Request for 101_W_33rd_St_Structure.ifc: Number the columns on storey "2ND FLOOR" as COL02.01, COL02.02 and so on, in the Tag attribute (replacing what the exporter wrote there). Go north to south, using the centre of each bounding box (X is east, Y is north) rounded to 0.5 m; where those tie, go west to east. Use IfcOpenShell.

First a look at what the model holds.

```python
import ifcopenshell
import ifcopenshell.util.element
import ifcopenshell.util.placement

model = ifcopenshell.open("101_W_33rd_St_Structure.ifc")
print(model.schema)
storey = next(s for s in model.by_type("IfcBuildingStorey") if s.Name == "2ND FLOOR")
columns = [e for e in ifcopenshell.util.element.get_decomposition(storey) if e.is_a("IfcColumn")]
for e in sorted(columns, key=lambda e: e.id()):
    origin = ifcopenshell.util.placement.get_local_placement(e.ObjectPlacement)[:3, 3]
    print(e.id(), e.Tag, e.Name, origin.round(2) + 0.0, sep=" | ")
```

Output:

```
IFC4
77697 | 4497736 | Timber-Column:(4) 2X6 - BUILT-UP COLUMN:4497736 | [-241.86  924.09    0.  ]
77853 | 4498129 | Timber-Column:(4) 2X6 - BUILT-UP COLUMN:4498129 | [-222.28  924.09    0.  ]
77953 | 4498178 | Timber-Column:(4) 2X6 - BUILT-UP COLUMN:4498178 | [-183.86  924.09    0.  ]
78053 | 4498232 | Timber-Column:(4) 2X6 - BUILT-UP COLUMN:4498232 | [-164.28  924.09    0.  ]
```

```python
import ifcopenshell
import ifcopenshell.geom
import ifcopenshell.util.element
import ifcopenshell.util.shape

model = ifcopenshell.open("101_W_33rd_St_Structure.ifc")
settings = ifcopenshell.geom.settings()
settings.set("use-world-coords", True)


def centre(element):
    shape = ifcopenshell.geom.create_shape(settings, element)
    return ifcopenshell.util.shape.get_bbox_centroid(shape.geometry)


storey = next(s for s in model.by_type("IfcBuildingStorey") if s.Name == "2ND FLOOR")
columns = [e for e in ifcopenshell.util.element.get_decomposition(storey) if e.is_a("IfcColumn")]

# Insertion points can sit at a corner or the storey origin, so sort by the geometry (in metres).
centres = {e: centre(e) for e in columns}
columns.sort(key=lambda e: (-round(centres[e][1] / 0.5), centres[e][0]))

for i, e in enumerate(columns, start=1):
    number = f"COL02.{i:02d}"
    e.Tag = number
    print(e.id(), number)

model.write("101_W_33rd_St_Structure_updated.ifc")
```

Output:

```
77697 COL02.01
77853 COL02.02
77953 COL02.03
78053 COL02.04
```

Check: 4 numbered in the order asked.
